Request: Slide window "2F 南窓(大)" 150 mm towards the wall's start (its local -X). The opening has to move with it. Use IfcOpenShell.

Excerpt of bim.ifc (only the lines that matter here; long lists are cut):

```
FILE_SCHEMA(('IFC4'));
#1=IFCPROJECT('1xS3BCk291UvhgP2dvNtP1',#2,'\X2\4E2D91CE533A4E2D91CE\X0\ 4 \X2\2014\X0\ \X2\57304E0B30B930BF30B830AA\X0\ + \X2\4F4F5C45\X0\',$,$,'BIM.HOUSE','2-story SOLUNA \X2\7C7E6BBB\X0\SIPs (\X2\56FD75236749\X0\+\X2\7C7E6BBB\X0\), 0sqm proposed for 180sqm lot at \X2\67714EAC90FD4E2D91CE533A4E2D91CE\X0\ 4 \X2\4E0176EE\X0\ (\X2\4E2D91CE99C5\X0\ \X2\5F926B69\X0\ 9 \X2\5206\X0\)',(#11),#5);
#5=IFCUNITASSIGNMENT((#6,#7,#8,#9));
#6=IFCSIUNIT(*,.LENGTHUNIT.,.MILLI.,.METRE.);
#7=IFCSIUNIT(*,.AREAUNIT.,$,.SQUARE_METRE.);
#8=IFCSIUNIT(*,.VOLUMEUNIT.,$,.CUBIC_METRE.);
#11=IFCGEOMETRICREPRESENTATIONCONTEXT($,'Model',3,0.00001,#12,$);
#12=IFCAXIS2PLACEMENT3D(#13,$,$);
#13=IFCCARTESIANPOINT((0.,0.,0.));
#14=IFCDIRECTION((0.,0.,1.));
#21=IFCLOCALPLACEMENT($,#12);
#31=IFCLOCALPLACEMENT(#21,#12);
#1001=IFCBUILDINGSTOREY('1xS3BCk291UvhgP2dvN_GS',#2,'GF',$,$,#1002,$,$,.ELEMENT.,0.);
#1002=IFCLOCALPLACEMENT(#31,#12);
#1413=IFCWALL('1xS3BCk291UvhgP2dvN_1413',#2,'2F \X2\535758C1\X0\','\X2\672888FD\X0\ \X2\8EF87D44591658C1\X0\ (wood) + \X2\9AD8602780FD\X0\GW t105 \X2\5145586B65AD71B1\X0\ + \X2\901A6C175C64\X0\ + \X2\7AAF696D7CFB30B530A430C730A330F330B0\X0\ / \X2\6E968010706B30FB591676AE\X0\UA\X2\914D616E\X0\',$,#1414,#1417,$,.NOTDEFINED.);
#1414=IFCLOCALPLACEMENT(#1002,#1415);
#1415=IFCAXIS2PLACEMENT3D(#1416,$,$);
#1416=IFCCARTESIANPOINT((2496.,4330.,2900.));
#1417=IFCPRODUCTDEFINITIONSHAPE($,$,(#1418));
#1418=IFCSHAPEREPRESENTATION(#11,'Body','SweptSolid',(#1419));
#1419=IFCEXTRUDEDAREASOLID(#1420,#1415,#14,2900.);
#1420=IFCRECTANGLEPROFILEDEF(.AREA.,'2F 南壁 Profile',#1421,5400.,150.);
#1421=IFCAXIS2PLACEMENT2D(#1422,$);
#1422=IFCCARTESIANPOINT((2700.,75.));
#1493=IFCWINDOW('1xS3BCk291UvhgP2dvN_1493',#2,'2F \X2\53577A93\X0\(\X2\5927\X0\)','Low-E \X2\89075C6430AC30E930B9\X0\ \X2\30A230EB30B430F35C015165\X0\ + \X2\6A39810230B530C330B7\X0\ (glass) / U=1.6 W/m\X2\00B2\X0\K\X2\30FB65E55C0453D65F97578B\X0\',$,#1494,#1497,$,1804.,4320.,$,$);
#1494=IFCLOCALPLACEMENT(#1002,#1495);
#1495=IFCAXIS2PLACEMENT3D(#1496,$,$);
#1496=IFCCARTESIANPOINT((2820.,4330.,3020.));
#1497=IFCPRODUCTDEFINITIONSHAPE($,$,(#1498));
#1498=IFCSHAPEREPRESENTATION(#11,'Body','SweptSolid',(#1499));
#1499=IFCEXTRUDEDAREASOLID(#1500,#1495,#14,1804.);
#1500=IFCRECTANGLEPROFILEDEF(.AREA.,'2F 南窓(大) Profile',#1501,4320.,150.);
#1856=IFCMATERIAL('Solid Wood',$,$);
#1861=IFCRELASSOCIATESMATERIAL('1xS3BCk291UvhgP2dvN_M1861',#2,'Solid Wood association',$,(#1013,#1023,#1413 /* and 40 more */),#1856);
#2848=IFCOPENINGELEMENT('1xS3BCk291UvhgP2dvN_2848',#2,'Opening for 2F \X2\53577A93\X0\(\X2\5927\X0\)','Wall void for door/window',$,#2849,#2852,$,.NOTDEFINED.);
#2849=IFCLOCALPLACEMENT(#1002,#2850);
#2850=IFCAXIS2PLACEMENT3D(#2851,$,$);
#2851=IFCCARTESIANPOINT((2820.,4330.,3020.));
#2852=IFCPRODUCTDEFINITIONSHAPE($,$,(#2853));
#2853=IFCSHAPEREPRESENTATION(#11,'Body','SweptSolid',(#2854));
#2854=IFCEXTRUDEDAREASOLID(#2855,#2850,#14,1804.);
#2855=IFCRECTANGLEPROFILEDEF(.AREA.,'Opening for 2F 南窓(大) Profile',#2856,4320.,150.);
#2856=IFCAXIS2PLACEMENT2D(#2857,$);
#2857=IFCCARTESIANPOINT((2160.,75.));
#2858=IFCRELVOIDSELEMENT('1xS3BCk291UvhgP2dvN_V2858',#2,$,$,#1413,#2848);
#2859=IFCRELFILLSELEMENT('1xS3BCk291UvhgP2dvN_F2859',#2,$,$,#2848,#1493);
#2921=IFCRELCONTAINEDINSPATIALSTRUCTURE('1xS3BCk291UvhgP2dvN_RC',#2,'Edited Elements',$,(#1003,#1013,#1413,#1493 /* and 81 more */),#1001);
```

```python
import ifcopenshell
import ifcopenshell.api.geometry
import ifcopenshell.util.placement

model = ifcopenshell.open("bim.ifc")

window = model.by_guid("1xS3BCk291UvhgP2dvN_1493")
opening = window.FillsVoids[0].RelatingOpeningElement
wall = opening.VoidsElements[0].RelatingBuildingElement

wall_matrix = ifcopenshell.util.placement.get_local_placement(wall.ObjectPlacement)
shift = wall_matrix[:3, 0] * -150.0
before = ifcopenshell.util.placement.get_local_placement(window.ObjectPlacement)[:3, 3].copy()

# The window is not placed relative to its opening, so move both.
for product in (opening, window):
    matrix = ifcopenshell.util.placement.get_local_placement(product.ObjectPlacement)
    matrix[:3, 3] += shift
    ifcopenshell.api.geometry.edit_object_placement(model, product=product, matrix=matrix, is_si=False)

after = ifcopenshell.util.placement.get_local_placement(window.ObjectPlacement)[:3, 3]
print("window moved by", (after - before).round(3) + 0.0)

model.write("bim_edited.ifc")
```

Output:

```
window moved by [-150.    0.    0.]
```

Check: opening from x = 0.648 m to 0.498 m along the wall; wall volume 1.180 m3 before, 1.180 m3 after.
